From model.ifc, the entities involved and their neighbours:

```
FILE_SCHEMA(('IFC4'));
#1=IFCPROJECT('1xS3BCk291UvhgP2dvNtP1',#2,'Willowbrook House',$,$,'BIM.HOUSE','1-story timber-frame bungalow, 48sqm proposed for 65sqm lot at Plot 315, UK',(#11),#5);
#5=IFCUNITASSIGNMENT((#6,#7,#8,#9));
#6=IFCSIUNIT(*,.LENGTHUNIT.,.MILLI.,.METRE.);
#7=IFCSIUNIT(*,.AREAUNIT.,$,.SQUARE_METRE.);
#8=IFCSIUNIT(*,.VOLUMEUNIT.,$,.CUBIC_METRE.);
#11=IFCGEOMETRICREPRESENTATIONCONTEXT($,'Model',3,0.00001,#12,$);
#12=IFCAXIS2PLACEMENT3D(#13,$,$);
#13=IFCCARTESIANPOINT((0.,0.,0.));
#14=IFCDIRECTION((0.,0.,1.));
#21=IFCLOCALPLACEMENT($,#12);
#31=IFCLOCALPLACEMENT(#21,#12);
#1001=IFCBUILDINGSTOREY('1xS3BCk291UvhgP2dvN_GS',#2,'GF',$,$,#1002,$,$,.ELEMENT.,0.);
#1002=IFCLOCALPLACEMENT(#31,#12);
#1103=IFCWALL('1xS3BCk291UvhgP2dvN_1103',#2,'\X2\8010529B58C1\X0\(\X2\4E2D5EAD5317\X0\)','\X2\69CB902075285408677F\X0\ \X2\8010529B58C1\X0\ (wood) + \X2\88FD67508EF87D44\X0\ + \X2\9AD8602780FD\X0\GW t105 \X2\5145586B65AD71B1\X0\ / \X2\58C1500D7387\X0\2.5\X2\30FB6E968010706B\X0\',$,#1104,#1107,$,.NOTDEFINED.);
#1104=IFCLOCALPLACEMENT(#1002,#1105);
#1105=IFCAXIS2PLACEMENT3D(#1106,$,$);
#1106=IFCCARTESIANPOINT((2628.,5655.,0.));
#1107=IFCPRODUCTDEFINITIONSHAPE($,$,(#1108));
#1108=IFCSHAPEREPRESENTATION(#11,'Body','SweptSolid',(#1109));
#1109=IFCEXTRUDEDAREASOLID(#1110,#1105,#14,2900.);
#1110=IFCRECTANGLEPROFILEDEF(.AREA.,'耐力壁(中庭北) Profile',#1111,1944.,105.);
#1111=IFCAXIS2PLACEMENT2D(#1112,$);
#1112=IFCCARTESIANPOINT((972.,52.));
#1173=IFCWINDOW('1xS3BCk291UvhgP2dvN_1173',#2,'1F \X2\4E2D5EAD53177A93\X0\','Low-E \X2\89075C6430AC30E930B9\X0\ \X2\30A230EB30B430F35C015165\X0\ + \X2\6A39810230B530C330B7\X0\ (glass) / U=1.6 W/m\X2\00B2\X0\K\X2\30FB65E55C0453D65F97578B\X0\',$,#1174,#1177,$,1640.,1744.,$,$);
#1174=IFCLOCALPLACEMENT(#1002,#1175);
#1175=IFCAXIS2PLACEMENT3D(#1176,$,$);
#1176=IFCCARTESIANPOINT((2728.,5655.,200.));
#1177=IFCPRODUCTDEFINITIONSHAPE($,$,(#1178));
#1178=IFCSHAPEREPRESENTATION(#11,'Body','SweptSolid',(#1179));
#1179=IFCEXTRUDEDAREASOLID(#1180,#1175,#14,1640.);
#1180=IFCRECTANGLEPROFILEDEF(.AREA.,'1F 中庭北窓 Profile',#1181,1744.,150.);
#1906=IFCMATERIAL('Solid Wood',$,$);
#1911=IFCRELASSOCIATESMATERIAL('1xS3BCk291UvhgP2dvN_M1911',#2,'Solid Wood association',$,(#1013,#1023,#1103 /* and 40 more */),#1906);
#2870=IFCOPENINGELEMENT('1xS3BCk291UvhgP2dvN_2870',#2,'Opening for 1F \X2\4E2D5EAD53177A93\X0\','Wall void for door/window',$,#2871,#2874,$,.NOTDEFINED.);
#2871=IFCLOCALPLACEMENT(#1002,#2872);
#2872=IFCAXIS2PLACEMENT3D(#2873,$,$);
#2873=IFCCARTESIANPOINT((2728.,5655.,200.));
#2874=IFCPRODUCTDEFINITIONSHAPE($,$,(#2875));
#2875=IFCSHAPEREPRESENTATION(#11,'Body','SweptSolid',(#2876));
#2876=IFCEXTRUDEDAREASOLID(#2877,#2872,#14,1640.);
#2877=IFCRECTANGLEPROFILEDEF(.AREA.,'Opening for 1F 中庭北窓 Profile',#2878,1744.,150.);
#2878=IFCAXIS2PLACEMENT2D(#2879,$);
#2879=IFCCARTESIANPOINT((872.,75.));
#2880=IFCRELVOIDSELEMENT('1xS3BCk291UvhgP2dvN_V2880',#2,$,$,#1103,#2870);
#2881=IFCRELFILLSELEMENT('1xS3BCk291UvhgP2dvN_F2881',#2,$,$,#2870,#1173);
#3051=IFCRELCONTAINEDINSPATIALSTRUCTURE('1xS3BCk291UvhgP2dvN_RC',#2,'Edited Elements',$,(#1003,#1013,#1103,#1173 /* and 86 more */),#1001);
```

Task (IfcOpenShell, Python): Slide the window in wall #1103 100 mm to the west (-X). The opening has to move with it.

```python
import ifcopenshell
import ifcopenshell.api.geometry
import ifcopenshell.util.placement
import ifcopenshell.util.unit

model = ifcopenshell.open("model.ifc")
unit_scale = ifcopenshell.util.unit.calculate_unit_scale(model)

window = model.by_id(1173)
opening = window.FillsVoids[0].RelatingOpeningElement
wall = opening.VoidsElements[0].RelatingBuildingElement

wall_matrix = ifcopenshell.util.placement.get_local_placement(wall.ObjectPlacement)
shift = wall_matrix[:3, 0] * -0.1 / unit_scale
before = ifcopenshell.util.placement.get_local_placement(window.ObjectPlacement)[:3, 3].copy()

# The window is not placed relative to its opening, so move both.
for product in (opening, window):
    matrix = ifcopenshell.util.placement.get_local_placement(product.ObjectPlacement)
    matrix[:3, 3] += shift
    ifcopenshell.api.geometry.edit_object_placement(model, product=product, matrix=matrix, is_si=False)

after = ifcopenshell.util.placement.get_local_placement(window.ObjectPlacement)[:3, 3]
print("window moved by", (after - before).round(3) + 0.0)

model.write("model_rev.ifc")
```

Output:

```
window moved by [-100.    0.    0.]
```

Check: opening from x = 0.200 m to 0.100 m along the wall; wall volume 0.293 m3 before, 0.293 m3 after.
